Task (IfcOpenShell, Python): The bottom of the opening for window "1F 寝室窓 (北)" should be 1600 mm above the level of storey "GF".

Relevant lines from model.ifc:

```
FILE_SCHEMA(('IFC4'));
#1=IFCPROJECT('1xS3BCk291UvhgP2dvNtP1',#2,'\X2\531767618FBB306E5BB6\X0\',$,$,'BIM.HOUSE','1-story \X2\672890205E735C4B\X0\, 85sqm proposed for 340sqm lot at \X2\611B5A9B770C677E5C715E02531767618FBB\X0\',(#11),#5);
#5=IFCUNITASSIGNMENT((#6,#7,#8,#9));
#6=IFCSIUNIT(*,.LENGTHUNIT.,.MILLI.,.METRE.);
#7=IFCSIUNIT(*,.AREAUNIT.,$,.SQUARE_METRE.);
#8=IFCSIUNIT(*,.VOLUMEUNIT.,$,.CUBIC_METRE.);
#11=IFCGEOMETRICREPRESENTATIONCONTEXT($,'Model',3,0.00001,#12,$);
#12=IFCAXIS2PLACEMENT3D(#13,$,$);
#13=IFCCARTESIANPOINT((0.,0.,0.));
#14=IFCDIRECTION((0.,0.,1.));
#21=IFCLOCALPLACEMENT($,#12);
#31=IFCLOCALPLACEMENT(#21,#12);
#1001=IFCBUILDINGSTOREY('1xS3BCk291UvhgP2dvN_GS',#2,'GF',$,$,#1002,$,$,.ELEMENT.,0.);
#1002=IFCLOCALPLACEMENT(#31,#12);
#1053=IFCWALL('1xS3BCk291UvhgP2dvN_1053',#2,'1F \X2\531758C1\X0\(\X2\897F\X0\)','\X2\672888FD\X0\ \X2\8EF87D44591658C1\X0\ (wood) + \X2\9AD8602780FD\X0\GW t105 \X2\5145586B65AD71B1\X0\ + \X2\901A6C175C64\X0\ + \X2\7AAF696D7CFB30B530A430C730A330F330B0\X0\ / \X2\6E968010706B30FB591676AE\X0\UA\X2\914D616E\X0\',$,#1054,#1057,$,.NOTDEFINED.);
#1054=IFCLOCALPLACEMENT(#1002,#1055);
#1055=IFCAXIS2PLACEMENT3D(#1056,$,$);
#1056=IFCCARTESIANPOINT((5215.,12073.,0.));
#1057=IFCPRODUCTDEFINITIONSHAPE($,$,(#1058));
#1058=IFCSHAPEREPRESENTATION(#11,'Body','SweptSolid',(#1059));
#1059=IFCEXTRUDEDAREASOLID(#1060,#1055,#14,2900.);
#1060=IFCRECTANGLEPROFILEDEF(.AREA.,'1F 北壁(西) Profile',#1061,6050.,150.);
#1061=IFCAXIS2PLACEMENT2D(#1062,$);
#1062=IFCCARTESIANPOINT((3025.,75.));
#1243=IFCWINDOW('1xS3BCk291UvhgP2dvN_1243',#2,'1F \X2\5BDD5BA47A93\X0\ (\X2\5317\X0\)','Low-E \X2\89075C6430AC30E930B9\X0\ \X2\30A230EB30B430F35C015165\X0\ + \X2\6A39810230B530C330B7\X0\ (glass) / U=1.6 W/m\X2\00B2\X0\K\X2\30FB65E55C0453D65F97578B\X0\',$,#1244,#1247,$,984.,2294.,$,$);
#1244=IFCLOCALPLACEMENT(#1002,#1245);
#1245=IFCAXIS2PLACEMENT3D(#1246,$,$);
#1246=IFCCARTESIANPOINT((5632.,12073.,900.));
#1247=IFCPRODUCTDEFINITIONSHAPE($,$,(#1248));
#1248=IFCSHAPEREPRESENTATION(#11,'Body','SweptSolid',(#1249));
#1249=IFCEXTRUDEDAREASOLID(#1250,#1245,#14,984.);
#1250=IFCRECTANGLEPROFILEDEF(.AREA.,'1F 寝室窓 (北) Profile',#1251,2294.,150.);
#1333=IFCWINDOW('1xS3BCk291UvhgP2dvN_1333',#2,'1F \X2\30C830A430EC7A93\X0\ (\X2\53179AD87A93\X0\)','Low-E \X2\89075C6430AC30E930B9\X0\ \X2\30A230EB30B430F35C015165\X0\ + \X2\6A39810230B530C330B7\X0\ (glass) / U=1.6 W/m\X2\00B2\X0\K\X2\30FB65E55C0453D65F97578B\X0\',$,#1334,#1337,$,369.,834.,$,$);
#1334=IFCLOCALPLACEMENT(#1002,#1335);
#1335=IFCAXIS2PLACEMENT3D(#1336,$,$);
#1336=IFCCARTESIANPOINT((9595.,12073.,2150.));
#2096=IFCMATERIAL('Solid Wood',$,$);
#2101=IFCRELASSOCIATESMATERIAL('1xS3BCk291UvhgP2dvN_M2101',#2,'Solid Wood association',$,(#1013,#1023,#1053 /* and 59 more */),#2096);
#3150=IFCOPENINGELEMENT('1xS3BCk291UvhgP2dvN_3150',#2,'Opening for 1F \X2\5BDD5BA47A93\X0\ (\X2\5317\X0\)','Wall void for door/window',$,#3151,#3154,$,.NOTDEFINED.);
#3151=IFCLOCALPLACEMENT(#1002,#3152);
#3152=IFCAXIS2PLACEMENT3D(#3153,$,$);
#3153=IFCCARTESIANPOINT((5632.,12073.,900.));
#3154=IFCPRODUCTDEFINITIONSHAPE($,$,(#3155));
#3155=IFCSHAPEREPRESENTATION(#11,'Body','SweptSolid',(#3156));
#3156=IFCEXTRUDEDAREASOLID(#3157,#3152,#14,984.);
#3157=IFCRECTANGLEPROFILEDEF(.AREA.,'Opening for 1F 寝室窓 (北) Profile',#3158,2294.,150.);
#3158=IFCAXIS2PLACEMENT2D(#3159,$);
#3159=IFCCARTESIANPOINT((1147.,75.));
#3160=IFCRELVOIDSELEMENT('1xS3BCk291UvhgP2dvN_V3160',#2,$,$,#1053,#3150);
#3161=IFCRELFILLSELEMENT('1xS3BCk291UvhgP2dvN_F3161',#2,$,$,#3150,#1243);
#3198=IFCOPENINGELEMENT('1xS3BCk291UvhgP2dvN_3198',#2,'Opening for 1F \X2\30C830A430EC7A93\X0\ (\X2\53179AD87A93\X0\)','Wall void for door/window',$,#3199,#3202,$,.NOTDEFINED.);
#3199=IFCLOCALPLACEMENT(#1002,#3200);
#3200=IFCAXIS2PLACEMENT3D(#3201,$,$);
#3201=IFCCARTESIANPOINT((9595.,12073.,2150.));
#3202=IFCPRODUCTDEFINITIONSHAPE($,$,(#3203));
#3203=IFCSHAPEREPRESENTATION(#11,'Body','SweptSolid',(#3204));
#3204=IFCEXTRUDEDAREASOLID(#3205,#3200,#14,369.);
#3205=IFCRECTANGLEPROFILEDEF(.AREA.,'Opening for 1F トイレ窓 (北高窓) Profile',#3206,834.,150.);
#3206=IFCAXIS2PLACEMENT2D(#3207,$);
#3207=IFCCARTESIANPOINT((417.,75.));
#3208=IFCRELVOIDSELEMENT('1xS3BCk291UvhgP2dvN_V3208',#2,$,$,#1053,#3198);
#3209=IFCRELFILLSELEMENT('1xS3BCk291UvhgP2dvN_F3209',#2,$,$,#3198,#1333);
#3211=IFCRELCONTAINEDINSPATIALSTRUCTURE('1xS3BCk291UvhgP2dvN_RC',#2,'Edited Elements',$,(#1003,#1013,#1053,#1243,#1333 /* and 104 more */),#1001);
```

```python
import numpy as np
import ifcopenshell
import ifcopenshell.api.geometry
import ifcopenshell.geom
import ifcopenshell.util.element
import ifcopenshell.util.placement
import ifcopenshell.util.shape
import ifcopenshell.util.unit

model = ifcopenshell.open("model.ifc")
unit_scale = ifcopenshell.util.unit.calculate_unit_scale(model)

window = model.by_guid("1xS3BCk291UvhgP2dvN_1243")
opening = window.FillsVoids[0].RelatingOpeningElement
storey = ifcopenshell.util.element.get_container(window, ifc_class="IfcBuildingStorey")
level = ifcopenshell.util.placement.get_local_placement(storey.ObjectPlacement)[2, 3]

# The opening's origin need not be at the sill, so measure its lowest point.
shape = ifcopenshell.geom.create_shape(ifcopenshell.geom.settings(), opening)
bottom = ifcopenshell.util.shape.get_shape_bottom_elevation(shape, shape.geometry) / unit_scale
dz = level + 1.6 / unit_scale - bottom

shift = np.array([0.0, 0.0, dz])
# The window is not placed relative to its opening, so move both.
for product in (opening, window):
    matrix = ifcopenshell.util.placement.get_local_placement(product.ObjectPlacement)
    matrix[:3, 3] += shift
    ifcopenshell.api.geometry.edit_object_placement(model, product=product, matrix=matrix, is_si=False)

print(f"moved by {dz * unit_scale:+.3f} m")

model.write("model_v2.ifc")
```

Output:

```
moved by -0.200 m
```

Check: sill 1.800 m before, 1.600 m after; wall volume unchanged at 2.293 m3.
